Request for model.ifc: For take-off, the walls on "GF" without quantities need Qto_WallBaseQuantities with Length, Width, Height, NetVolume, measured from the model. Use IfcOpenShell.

First a look at what the model holds.

```python
import ifcopenshell
import ifcopenshell.util.element
import ifcopenshell.util.unit

model = ifcopenshell.open("model.ifc")
print(model.schema)
for unit_type in ("LENGTHUNIT", "AREAUNIT", "VOLUMEUNIT"):
    print(unit_type, ifcopenshell.util.unit.calculate_unit_scale(model, unit_type))
storey = next(s for s in model.by_type("IfcBuildingStorey") if s.Name == "GF")
walls = [e for e in ifcopenshell.util.element.get_decomposition(storey) if e.is_a("IfcWall")]
for e in sorted(walls, key=lambda e: e.id()):
    print(e.id(), e.is_a(), e.Name, list(ifcopenshell.util.element.get_psets(e, qtos_only=True)), sep=" | ")
```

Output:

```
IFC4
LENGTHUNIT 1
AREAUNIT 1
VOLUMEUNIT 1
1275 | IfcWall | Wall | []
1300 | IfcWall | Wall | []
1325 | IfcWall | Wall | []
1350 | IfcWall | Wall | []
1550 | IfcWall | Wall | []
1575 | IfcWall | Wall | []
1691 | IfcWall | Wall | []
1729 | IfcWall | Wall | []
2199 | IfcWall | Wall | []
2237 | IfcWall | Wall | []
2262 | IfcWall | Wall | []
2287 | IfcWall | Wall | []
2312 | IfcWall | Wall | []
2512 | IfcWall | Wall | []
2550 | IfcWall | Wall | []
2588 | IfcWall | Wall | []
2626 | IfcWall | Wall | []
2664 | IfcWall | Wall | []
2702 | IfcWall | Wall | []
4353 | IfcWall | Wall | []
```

```python
import ifcopenshell
import ifcopenshell.api.pset
import ifcopenshell.geom
import ifcopenshell.util.element
import ifcopenshell.util.shape
import ifcopenshell.util.unit

model = ifcopenshell.open("model.ifc")
unit_scale = ifcopenshell.util.unit.calculate_unit_scale(model)
volume_scale = ifcopenshell.util.unit.calculate_unit_scale(model, "VOLUMEUNIT")
settings = ifcopenshell.geom.settings()

storey = next(s for s in model.by_type("IfcBuildingStorey") if s.Name == "GF")
walls = [e for e in ifcopenshell.util.element.get_decomposition(storey) if e.is_a("IfcWall")]

for e in sorted(walls, key=lambda e: e.id()):
    if ifcopenshell.util.element.get_psets(e, qtos_only=True, should_inherit=False):
        continue
    # Geometry comes back in metres, in the element's own axes.
    shape = ifcopenshell.geom.create_shape(settings, e)
    values = {
        "Length": ifcopenshell.util.shape.get_x(shape.geometry) / unit_scale,
        "Width": ifcopenshell.util.shape.get_y(shape.geometry) / unit_scale,
        "Height": ifcopenshell.util.shape.get_z(shape.geometry) / unit_scale,
        "NetVolume": ifcopenshell.util.shape.get_volume(shape.geometry) / volume_scale,
    }
    qto = ifcopenshell.api.pset.add_qto(model, product=e, name="Qto_WallBaseQuantities")
    ifcopenshell.api.pset.edit_qto(model, qto=qto, properties=values)
    print(e.id(), {k: round(v, 3) for k, v in values.items()})

model.write("model_edited.ifc")
```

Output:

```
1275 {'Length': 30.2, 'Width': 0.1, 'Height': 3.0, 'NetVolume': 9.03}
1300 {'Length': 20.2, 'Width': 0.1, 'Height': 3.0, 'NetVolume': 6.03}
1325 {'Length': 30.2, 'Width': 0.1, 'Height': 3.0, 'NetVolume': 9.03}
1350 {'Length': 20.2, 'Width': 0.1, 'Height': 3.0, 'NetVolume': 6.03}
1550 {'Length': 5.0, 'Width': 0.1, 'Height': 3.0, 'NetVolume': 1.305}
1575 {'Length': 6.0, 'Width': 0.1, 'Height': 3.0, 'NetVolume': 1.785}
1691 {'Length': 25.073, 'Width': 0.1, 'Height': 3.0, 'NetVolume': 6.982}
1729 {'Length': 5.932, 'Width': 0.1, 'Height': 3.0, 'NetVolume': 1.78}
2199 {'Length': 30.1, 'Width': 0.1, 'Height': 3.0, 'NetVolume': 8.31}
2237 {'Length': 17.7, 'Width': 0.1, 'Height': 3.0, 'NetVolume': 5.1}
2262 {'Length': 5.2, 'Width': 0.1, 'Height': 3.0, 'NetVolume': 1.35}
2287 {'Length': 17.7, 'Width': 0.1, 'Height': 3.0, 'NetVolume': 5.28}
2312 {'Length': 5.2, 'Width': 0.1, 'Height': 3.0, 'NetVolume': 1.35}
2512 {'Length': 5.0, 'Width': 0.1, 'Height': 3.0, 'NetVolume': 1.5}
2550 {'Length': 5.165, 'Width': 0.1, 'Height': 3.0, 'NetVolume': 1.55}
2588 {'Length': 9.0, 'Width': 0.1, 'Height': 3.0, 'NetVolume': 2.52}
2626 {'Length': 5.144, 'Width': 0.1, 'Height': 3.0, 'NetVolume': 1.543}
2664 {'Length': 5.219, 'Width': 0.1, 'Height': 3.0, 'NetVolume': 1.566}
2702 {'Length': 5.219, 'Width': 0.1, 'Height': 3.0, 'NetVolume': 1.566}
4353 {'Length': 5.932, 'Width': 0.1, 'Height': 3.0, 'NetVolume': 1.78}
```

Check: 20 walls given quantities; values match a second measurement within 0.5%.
